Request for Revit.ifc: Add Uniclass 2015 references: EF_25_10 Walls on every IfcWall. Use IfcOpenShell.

First a look at what the model holds.

```python
import ifcopenshell

model = ifcopenshell.open("Revit.ifc")
print(model.schema)
print("classifications:", [c.Name for c in model.by_type("IfcClassification")])
for ifc_class in ("IfcDoor", "IfcRoof", "IfcStair", "IfcWall", "IfcWindow"):
    print(ifc_class, len(model.by_type(ifc_class)))
```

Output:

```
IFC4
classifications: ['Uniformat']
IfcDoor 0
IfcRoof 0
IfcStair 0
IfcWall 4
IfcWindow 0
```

```python
import ifcopenshell
import ifcopenshell.api.classification

model = ifcopenshell.open("Revit.ifc")

system = ifcopenshell.api.classification.add_classification(model, classification="Uniclass 2015")

codes = {
    "IfcWall": ("EF_25_10", "Walls"),
}
for ifc_class, (code, name) in codes.items():
    products = model.by_type(ifc_class)
    ifcopenshell.api.classification.add_reference(
        model, products=products, classification=system, identification=code, name=name
    )
    print(code, len(products))

model.write("Revit_updated.ifc")
```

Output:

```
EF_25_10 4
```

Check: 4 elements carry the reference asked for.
